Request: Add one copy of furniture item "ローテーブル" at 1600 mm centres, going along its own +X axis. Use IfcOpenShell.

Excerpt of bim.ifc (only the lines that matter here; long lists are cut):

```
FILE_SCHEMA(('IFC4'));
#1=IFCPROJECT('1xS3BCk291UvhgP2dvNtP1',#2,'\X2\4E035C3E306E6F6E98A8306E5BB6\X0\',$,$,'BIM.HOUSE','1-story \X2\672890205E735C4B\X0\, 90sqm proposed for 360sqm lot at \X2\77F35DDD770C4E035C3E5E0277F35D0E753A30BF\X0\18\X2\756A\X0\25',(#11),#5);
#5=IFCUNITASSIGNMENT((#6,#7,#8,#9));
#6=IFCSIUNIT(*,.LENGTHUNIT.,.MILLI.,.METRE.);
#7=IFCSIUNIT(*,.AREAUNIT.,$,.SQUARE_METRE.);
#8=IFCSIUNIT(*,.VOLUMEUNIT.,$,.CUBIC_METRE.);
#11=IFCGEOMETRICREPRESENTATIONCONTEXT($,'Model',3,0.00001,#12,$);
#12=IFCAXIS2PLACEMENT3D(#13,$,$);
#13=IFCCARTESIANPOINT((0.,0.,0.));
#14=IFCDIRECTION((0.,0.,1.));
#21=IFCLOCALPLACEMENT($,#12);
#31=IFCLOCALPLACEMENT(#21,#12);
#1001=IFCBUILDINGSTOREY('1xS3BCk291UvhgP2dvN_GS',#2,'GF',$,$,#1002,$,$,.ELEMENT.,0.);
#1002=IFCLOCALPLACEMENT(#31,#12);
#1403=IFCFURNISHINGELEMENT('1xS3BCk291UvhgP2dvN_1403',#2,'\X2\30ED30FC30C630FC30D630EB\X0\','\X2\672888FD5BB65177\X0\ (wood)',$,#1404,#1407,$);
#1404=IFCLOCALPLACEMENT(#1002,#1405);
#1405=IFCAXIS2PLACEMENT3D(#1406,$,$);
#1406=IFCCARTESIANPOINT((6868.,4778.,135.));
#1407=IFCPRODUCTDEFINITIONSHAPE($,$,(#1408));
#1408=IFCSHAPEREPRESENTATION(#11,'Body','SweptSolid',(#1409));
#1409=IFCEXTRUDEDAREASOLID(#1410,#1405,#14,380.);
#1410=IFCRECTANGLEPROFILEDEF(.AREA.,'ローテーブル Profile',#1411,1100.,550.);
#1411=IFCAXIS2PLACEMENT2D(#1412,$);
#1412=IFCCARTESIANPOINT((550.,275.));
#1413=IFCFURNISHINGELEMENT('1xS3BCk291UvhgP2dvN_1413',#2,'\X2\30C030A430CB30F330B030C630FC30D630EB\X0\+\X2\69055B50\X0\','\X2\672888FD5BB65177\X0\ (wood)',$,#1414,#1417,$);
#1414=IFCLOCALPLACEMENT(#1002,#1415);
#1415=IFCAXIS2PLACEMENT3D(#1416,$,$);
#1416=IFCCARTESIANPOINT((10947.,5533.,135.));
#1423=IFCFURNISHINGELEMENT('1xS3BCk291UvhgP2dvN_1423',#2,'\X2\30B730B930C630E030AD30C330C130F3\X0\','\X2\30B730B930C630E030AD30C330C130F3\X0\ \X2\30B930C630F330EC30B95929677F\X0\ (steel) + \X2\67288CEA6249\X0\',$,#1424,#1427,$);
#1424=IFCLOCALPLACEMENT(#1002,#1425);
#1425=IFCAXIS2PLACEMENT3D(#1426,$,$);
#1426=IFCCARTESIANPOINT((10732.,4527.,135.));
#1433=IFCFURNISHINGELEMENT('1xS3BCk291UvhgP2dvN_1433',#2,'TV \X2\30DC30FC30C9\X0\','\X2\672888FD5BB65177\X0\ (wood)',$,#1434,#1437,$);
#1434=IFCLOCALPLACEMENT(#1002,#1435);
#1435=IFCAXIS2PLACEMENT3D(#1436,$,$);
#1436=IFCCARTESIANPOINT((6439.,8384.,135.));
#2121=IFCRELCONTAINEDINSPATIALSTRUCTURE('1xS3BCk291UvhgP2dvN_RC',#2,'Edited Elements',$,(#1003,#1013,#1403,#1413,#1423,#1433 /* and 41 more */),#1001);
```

```python
import ifcopenshell
import ifcopenshell.api.geometry
import ifcopenshell.api.root
import ifcopenshell.util.element
import ifcopenshell.util.placement
import ifcopenshell.util.unit

model = ifcopenshell.open("bim.ifc")
unit_scale = ifcopenshell.util.unit.calculate_unit_scale(model)


def reuse_history(source, copy):
    """copy_class also copies each property set's owner history, people and application; keep the originals."""
    for rel in copy.IsDefinedBy:
        if rel.is_a("IfcRelDefinesByProperties") and (history := rel.RelatingPropertyDefinition.OwnerHistory):
            rel.RelatingPropertyDefinition.OwnerHistory = source.OwnerHistory
            ifcopenshell.util.element.remove_deep2(model, history)


source = model.by_guid("1xS3BCk291UvhgP2dvN_1403")
base = ifcopenshell.util.placement.get_local_placement(source.ObjectPlacement)
step = base[:3, 0] * 1.6 / unit_scale

for i in range(1, 2):
    copy = ifcopenshell.api.root.copy_class(model, product=source)
    copy.Representation = ifcopenshell.util.element.copy_deep(
        model, source.Representation, exclude=["IfcGeometricRepresentationContext", "IfcRepresentationMap"]
    )
    reuse_history(source, copy)
    matrix = base.copy()
    matrix[:3, 3] += i * step
    print("added at", matrix[:3, 3].round(3) + 0.0)
    ifcopenshell.api.geometry.edit_object_placement(model, product=copy, matrix=matrix, is_si=False)

model.write("bim_edited.ifc")
```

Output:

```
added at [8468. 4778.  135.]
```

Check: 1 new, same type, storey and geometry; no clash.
